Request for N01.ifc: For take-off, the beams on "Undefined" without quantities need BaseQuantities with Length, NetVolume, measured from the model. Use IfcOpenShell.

First a look at what the model holds.

```python
import ifcopenshell
import ifcopenshell.util.element
import ifcopenshell.util.unit

model = ifcopenshell.open("N01.ifc")
print(model.schema)
for unit_type in ("LENGTHUNIT", "AREAUNIT", "VOLUMEUNIT"):
    print(unit_type, ifcopenshell.util.unit.calculate_unit_scale(model, unit_type))
storey = next(s for s in model.by_type("IfcBuildingStorey") if s.Name == "Undefined")
beams = [e for e in ifcopenshell.util.element.get_decomposition(storey) if e.is_a("IfcBeam")]
for e in sorted(beams, key=lambda e: e.id()):
    print(e.id(), e.is_a(), e.Name, list(ifcopenshell.util.element.get_psets(e, qtos_only=True)), sep=" | ")
```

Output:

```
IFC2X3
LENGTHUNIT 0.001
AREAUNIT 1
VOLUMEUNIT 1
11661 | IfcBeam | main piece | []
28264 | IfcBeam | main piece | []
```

```python
import ifcopenshell
import ifcopenshell.api.pset
import ifcopenshell.geom
import ifcopenshell.util.element
import ifcopenshell.util.shape
import ifcopenshell.util.unit

model = ifcopenshell.open("N01.ifc")
unit_scale = ifcopenshell.util.unit.calculate_unit_scale(model)
volume_scale = ifcopenshell.util.unit.calculate_unit_scale(model, "VOLUMEUNIT")
settings = ifcopenshell.geom.settings()

storey = next(s for s in model.by_type("IfcBuildingStorey") if s.Name == "Undefined")
beams = [e for e in ifcopenshell.util.element.get_decomposition(storey) if e.is_a("IfcBeam")]

for e in sorted(beams, key=lambda e: e.id()):
    if ifcopenshell.util.element.get_psets(e, qtos_only=True, should_inherit=False):
        continue
    # Geometry comes back in metres, in the element's own axes.
    shape = ifcopenshell.geom.create_shape(settings, e)
    values = {
        "Length": ifcopenshell.util.shape.get_max_xyz(shape.geometry) / unit_scale,
        "NetVolume": ifcopenshell.util.shape.get_volume(shape.geometry) / volume_scale,
    }
    qto = ifcopenshell.api.pset.add_qto(model, product=e, name="BaseQuantities")
    ifcopenshell.api.pset.edit_qto(model, qto=qto, properties=values)
    print(e.id(), {k: round(v, 3) for k, v in values.items()})

model.write("N01_v2.ifc")
```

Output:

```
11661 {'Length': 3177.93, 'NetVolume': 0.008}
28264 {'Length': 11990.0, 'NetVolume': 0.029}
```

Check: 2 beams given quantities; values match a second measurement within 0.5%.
